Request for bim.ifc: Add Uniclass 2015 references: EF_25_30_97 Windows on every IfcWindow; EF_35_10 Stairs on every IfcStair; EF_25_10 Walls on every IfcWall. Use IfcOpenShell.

First a look at what the model holds.

```python
import ifcopenshell

model = ifcopenshell.open("bim.ifc")
print(model.schema)
print("classifications:", [c.Name for c in model.by_type("IfcClassification")])
for ifc_class in ("IfcDoor", "IfcRoof", "IfcStair", "IfcWall", "IfcWindow"):
    print(ifc_class, len(model.by_type(ifc_class)))
```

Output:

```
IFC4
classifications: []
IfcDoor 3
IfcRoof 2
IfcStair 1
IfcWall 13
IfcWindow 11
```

```python
import ifcopenshell
import ifcopenshell.api.classification

model = ifcopenshell.open("bim.ifc")

system = ifcopenshell.api.classification.add_classification(model, classification="Uniclass 2015")

codes = {
    "IfcWindow": ("EF_25_30_97", "Windows"),
    "IfcStair": ("EF_35_10", "Stairs"),
    "IfcWall": ("EF_25_10", "Walls"),
}
for ifc_class, (code, name) in codes.items():
    products = model.by_type(ifc_class)
    ifcopenshell.api.classification.add_reference(
        model, products=products, classification=system, identification=code, name=name
    )
    print(code, len(products))

model.write("bim_updated.ifc")
```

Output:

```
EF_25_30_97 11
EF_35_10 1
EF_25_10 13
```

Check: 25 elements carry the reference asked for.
